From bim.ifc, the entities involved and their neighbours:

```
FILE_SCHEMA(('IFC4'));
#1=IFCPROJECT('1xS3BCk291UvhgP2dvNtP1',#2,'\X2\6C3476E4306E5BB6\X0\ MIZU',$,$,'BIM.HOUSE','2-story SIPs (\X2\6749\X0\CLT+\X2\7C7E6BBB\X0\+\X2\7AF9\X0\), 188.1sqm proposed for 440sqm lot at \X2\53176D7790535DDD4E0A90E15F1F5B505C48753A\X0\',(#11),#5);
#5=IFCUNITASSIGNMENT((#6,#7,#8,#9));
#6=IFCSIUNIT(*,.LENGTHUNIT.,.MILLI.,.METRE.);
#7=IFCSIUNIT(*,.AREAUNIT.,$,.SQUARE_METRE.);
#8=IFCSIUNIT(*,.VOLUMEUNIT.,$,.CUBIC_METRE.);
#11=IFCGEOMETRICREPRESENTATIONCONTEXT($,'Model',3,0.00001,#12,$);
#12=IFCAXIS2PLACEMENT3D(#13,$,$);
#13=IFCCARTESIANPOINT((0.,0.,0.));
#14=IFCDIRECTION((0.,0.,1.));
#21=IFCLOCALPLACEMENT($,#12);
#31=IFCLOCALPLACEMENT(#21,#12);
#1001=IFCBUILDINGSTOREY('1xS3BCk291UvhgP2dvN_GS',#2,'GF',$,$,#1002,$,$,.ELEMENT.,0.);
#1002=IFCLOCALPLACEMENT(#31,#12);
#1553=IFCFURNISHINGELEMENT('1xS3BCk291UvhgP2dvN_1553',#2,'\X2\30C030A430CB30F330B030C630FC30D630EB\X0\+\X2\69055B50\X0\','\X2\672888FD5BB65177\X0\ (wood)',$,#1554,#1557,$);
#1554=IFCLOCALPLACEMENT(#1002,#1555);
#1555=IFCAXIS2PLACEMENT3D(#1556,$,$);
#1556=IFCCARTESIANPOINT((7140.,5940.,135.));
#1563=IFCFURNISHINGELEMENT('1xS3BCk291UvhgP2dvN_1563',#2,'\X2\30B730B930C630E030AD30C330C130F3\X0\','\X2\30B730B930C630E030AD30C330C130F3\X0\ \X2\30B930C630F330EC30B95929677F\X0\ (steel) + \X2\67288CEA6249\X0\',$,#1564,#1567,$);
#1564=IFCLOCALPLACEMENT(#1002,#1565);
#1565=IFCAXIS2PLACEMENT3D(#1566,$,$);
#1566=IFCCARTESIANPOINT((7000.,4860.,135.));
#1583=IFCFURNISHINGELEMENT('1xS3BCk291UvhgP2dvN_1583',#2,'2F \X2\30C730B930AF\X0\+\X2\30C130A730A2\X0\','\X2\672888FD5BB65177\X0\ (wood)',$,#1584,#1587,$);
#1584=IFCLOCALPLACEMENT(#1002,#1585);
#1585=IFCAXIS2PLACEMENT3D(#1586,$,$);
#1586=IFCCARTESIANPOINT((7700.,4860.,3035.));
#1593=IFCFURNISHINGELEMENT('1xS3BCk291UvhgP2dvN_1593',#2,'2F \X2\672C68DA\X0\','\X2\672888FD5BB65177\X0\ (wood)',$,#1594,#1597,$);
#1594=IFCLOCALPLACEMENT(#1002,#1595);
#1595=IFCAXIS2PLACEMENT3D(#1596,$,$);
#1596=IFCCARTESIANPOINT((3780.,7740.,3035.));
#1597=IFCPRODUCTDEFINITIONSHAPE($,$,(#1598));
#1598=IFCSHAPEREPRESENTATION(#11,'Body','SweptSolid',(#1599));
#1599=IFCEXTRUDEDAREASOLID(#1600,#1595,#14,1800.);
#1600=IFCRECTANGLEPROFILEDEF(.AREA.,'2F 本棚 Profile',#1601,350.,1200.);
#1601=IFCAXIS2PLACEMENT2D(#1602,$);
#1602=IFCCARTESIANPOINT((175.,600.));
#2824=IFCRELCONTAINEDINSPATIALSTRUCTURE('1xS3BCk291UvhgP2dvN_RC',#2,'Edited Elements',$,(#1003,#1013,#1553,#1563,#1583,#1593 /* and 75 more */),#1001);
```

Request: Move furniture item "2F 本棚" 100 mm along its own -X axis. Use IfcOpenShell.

```python
import ifcopenshell
import ifcopenshell.api.geometry
import ifcopenshell.util.placement
import ifcopenshell.util.unit

model = ifcopenshell.open("bim.ifc")
unit_scale = ifcopenshell.util.unit.calculate_unit_scale(model)

item = model.by_id(1593)
matrix = ifcopenshell.util.placement.get_local_placement(item.ObjectPlacement)
matrix[:3, 3] -= matrix[:3, 0] * 0.1 / unit_scale
ifcopenshell.api.geometry.edit_object_placement(model, product=item, matrix=matrix, is_si=False)

print(ifcopenshell.util.placement.get_local_placement(item.ObjectPlacement).round(3) + 0.0)

model.write("bim_updated.ifc")
```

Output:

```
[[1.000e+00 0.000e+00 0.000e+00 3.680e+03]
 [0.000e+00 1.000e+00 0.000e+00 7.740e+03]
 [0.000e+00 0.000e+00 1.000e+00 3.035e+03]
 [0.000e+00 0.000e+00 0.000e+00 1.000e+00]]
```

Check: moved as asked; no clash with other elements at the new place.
